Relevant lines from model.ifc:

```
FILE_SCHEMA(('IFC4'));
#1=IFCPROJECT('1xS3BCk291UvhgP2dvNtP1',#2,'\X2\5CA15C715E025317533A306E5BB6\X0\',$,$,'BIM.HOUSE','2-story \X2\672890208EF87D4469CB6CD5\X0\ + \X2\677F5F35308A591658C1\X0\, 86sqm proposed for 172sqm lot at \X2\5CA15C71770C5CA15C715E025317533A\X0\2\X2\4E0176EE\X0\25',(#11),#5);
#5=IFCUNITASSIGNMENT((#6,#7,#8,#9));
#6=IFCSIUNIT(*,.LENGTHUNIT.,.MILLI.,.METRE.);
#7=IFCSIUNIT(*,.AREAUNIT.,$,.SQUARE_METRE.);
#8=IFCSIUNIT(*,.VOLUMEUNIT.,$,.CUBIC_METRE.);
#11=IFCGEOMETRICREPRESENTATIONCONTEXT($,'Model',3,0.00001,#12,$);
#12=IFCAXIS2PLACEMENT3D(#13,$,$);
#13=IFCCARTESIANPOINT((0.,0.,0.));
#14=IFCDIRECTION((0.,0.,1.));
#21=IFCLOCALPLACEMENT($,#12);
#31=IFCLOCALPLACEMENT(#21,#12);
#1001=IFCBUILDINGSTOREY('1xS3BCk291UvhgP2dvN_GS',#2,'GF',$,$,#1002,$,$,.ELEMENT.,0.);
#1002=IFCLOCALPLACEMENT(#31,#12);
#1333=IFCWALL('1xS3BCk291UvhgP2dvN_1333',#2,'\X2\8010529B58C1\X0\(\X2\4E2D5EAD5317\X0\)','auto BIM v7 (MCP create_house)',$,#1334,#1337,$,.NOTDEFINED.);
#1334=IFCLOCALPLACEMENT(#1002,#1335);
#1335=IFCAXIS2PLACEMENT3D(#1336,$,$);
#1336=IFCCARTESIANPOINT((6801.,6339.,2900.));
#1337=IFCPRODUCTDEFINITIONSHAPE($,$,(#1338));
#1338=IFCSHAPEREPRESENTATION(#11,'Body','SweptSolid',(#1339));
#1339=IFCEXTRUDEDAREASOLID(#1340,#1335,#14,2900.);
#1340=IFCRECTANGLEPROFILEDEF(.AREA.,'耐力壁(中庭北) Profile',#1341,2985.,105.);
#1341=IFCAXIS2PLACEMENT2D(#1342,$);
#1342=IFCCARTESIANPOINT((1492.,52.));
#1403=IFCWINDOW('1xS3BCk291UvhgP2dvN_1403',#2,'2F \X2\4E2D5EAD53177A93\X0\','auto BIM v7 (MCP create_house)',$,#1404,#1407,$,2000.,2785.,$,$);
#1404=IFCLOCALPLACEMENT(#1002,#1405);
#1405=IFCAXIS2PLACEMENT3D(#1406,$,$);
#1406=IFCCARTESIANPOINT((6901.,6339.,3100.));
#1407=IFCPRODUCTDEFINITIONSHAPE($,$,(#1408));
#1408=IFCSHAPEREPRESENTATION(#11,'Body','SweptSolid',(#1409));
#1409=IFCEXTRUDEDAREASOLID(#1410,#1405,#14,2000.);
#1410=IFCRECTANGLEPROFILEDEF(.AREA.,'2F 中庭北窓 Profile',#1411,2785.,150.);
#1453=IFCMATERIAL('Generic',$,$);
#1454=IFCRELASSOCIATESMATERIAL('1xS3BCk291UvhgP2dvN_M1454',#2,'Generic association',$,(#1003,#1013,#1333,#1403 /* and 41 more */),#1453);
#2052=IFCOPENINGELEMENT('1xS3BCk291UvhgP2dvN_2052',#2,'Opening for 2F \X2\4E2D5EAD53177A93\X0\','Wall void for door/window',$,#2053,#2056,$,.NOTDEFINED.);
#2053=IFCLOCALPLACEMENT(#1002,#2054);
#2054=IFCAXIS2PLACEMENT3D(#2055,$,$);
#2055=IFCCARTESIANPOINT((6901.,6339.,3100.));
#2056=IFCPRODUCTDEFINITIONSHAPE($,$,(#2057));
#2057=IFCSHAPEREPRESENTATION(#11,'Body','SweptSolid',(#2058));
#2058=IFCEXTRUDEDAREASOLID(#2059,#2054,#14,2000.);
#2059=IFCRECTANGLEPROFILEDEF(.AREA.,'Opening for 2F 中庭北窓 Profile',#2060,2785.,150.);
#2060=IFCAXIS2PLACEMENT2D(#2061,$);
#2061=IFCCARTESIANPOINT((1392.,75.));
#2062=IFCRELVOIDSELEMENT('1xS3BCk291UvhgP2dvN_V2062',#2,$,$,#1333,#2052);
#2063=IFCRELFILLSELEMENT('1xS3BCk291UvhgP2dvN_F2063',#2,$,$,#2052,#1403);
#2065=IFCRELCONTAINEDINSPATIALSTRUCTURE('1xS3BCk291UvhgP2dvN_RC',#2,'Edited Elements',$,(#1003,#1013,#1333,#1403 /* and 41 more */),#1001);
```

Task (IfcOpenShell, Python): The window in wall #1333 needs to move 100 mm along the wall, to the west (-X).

```python
import ifcopenshell
import ifcopenshell.api.geometry
import ifcopenshell.util.placement
import ifcopenshell.util.unit

model = ifcopenshell.open("model.ifc")
unit_scale = ifcopenshell.util.unit.calculate_unit_scale(model)

window = model.by_guid("1xS3BCk291UvhgP2dvN_1403")
opening = window.FillsVoids[0].RelatingOpeningElement
wall = opening.VoidsElements[0].RelatingBuildingElement

wall_matrix = ifcopenshell.util.placement.get_local_placement(wall.ObjectPlacement)
shift = wall_matrix[:3, 0] * -0.1 / unit_scale
before = ifcopenshell.util.placement.get_local_placement(window.ObjectPlacement)[:3, 3].copy()

# The window is not placed relative to its opening, so move both.
for product in (opening, window):
    matrix = ifcopenshell.util.placement.get_local_placement(product.ObjectPlacement)
    matrix[:3, 3] += shift
    ifcopenshell.api.geometry.edit_object_placement(model, product=product, matrix=matrix, is_si=False)

after = ifcopenshell.util.placement.get_local_placement(window.ObjectPlacement)[:3, 3]
print("window moved by", (after - before).round(3) + 0.0)

model.write("model_rev.ifc")
```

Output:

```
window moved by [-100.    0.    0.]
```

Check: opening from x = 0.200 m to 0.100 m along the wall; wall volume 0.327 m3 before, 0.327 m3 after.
